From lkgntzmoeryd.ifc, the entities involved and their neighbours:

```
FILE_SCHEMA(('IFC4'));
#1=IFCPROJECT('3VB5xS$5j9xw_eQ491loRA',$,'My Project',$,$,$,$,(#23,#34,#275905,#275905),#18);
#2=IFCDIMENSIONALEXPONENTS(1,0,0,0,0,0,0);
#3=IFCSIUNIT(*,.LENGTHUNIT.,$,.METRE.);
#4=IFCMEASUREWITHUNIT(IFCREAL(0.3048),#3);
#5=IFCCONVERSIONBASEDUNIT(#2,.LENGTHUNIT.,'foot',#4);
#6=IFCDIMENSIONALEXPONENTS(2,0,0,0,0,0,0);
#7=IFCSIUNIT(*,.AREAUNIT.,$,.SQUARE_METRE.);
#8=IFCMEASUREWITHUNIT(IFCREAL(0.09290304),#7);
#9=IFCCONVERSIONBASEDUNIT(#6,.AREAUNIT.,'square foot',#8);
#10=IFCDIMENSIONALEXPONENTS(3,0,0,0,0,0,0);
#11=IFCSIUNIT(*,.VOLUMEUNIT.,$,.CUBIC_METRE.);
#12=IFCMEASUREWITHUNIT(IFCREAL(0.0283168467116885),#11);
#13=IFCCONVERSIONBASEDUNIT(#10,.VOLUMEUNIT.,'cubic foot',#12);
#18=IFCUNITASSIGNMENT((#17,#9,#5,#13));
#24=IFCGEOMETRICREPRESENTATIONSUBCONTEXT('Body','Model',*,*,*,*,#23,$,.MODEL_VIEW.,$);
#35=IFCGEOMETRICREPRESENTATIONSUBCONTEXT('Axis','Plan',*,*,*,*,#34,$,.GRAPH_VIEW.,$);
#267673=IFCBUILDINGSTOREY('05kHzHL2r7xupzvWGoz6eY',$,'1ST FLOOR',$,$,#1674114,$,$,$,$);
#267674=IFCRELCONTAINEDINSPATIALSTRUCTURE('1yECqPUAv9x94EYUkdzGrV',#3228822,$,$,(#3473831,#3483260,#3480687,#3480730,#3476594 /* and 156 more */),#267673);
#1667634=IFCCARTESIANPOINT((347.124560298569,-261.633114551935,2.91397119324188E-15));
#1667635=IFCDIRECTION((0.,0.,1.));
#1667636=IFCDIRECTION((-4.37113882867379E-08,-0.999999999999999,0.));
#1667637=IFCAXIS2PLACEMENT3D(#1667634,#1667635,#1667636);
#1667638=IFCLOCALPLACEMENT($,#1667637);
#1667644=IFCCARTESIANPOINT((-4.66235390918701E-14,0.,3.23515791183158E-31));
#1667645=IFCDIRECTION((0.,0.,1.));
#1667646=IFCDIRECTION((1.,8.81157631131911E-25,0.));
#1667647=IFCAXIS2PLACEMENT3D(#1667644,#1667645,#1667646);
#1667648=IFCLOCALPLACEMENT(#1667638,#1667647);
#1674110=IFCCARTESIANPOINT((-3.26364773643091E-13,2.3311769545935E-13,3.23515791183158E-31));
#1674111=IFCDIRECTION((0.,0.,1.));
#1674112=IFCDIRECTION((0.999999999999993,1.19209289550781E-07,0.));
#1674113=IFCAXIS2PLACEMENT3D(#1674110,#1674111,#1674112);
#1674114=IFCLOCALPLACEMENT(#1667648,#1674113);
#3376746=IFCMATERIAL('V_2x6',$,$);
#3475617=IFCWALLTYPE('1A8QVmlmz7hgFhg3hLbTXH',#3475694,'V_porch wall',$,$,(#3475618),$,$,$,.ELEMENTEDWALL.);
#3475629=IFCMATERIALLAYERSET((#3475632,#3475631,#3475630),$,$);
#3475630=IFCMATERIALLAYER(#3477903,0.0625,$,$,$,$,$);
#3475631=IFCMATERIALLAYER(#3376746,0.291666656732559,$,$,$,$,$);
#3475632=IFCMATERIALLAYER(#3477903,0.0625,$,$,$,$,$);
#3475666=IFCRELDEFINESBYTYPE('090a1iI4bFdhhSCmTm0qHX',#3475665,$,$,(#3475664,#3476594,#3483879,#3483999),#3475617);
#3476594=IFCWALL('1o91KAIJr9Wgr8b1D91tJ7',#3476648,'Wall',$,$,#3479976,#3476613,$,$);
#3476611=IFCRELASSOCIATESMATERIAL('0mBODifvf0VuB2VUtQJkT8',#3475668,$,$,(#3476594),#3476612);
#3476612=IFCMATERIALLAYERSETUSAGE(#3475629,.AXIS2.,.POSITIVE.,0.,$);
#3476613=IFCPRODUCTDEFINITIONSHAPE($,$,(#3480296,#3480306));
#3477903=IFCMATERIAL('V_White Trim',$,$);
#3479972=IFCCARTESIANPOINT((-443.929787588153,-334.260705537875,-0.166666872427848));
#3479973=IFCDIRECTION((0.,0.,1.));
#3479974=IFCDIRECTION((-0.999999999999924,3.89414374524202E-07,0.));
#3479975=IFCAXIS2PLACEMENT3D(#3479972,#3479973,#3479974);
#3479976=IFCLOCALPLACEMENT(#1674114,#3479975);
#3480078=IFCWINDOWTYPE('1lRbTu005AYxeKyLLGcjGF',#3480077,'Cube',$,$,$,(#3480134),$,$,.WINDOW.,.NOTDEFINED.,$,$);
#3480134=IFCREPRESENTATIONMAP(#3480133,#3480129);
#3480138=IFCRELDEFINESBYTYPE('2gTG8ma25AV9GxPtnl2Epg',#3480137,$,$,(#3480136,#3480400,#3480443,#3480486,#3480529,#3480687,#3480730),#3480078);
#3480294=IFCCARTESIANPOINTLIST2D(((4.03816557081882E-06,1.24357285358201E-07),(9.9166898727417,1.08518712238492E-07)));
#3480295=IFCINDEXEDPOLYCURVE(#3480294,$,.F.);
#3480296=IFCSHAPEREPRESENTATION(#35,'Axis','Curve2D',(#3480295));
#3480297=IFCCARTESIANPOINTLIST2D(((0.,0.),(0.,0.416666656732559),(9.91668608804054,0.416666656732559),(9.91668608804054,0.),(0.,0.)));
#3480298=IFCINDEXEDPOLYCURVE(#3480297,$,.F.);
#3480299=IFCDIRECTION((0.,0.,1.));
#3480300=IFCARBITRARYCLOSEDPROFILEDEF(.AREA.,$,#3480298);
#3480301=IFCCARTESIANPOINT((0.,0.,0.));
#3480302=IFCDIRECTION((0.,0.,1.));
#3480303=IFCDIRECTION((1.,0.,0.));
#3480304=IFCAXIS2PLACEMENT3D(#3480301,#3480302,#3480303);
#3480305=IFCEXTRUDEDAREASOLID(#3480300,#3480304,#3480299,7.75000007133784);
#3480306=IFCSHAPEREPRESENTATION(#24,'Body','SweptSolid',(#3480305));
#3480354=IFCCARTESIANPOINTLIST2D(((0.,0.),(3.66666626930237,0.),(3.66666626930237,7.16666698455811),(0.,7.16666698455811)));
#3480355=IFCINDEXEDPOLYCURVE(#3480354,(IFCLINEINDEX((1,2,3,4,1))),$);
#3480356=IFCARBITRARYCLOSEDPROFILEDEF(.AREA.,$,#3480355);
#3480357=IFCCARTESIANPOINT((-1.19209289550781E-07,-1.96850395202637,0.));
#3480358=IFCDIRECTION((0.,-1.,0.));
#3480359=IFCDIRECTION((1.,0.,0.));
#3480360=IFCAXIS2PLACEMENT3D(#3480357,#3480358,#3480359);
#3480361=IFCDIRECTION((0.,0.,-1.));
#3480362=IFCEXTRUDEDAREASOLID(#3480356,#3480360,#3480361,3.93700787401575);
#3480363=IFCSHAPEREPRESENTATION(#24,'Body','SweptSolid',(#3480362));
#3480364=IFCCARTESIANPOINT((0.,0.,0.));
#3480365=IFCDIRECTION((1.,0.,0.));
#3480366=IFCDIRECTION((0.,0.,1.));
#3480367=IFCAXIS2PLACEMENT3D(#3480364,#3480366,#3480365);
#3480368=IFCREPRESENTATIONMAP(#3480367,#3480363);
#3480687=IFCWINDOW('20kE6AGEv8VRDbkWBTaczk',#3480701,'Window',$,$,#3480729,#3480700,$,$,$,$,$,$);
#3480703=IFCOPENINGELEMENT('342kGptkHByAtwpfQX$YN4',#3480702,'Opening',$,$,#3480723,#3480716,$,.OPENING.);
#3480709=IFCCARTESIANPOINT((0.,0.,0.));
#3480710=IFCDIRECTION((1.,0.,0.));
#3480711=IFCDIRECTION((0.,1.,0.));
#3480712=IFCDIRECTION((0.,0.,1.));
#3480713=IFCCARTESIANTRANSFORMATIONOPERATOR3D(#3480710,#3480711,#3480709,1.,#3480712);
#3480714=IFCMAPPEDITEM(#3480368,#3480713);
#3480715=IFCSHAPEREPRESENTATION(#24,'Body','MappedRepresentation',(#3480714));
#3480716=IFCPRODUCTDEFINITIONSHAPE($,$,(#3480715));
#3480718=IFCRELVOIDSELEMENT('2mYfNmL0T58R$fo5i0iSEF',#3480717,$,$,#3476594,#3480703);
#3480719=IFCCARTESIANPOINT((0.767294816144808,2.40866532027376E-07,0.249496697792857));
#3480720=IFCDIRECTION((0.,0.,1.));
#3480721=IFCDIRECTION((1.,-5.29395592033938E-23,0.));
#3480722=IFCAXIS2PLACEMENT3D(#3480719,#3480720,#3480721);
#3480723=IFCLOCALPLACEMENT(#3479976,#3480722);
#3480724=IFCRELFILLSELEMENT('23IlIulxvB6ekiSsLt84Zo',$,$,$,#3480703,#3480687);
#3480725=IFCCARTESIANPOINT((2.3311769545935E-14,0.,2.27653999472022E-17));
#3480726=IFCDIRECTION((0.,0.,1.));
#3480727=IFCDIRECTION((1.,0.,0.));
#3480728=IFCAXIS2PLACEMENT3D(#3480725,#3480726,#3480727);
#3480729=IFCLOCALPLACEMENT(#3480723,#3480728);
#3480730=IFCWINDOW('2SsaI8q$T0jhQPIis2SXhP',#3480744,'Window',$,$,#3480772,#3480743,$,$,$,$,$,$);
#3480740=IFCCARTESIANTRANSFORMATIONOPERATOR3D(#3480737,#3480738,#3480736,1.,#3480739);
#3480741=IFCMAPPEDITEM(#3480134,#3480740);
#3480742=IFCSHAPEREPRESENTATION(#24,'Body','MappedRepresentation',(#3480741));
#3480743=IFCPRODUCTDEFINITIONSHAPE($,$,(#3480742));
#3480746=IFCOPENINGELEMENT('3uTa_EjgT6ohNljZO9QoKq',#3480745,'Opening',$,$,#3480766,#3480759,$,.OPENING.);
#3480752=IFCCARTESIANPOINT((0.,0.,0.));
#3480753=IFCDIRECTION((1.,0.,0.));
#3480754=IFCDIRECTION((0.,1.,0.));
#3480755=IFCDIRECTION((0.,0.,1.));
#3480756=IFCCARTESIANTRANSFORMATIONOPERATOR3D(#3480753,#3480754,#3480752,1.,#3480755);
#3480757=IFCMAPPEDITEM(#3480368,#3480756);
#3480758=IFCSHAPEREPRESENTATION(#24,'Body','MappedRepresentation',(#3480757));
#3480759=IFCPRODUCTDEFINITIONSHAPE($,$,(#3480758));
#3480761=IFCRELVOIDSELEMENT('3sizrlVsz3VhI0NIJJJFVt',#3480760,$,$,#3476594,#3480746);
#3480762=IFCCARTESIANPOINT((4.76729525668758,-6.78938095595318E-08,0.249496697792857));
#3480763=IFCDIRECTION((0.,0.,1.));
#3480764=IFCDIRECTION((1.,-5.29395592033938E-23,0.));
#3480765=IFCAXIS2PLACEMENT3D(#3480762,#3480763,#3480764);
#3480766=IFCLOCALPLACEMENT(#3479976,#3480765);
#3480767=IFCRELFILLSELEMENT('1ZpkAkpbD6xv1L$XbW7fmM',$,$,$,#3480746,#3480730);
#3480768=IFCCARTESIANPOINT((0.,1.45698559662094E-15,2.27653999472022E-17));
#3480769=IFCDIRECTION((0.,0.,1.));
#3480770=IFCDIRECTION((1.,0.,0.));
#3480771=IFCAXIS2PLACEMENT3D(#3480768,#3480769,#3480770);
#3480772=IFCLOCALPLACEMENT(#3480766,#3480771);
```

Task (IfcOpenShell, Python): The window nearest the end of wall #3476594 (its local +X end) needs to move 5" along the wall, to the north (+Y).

```python
import ifcopenshell
import ifcopenshell.api.geometry
import ifcopenshell.util.placement
import ifcopenshell.util.unit

model = ifcopenshell.open("lkgntzmoeryd.ifc")
unit_scale = ifcopenshell.util.unit.calculate_unit_scale(model)

window = model.by_id(3480730)
opening = window.FillsVoids[0].RelatingOpeningElement
wall = opening.VoidsElements[0].RelatingBuildingElement

wall_matrix = ifcopenshell.util.placement.get_local_placement(wall.ObjectPlacement)
shift = wall_matrix[:3, 0] * 5 * 0.0254 / unit_scale
before = ifcopenshell.util.placement.get_local_placement(window.ObjectPlacement)[:3, 3].copy()

# The window is placed relative to its opening, so it follows when the opening moves.
matrix = ifcopenshell.util.placement.get_local_placement(opening.ObjectPlacement)
matrix[:3, 3] += shift
ifcopenshell.api.geometry.edit_object_placement(
    model, product=opening, matrix=matrix, is_si=False, should_transform_children=True
)

after = ifcopenshell.util.placement.get_local_placement(window.ObjectPlacement)[:3, 3]
print("window moved by", (after - before).round(3) + 0.0)

model.write("lkgntzmoeryd_updated.ifc")
```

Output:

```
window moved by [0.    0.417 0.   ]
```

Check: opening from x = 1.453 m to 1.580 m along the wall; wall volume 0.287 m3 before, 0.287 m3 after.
